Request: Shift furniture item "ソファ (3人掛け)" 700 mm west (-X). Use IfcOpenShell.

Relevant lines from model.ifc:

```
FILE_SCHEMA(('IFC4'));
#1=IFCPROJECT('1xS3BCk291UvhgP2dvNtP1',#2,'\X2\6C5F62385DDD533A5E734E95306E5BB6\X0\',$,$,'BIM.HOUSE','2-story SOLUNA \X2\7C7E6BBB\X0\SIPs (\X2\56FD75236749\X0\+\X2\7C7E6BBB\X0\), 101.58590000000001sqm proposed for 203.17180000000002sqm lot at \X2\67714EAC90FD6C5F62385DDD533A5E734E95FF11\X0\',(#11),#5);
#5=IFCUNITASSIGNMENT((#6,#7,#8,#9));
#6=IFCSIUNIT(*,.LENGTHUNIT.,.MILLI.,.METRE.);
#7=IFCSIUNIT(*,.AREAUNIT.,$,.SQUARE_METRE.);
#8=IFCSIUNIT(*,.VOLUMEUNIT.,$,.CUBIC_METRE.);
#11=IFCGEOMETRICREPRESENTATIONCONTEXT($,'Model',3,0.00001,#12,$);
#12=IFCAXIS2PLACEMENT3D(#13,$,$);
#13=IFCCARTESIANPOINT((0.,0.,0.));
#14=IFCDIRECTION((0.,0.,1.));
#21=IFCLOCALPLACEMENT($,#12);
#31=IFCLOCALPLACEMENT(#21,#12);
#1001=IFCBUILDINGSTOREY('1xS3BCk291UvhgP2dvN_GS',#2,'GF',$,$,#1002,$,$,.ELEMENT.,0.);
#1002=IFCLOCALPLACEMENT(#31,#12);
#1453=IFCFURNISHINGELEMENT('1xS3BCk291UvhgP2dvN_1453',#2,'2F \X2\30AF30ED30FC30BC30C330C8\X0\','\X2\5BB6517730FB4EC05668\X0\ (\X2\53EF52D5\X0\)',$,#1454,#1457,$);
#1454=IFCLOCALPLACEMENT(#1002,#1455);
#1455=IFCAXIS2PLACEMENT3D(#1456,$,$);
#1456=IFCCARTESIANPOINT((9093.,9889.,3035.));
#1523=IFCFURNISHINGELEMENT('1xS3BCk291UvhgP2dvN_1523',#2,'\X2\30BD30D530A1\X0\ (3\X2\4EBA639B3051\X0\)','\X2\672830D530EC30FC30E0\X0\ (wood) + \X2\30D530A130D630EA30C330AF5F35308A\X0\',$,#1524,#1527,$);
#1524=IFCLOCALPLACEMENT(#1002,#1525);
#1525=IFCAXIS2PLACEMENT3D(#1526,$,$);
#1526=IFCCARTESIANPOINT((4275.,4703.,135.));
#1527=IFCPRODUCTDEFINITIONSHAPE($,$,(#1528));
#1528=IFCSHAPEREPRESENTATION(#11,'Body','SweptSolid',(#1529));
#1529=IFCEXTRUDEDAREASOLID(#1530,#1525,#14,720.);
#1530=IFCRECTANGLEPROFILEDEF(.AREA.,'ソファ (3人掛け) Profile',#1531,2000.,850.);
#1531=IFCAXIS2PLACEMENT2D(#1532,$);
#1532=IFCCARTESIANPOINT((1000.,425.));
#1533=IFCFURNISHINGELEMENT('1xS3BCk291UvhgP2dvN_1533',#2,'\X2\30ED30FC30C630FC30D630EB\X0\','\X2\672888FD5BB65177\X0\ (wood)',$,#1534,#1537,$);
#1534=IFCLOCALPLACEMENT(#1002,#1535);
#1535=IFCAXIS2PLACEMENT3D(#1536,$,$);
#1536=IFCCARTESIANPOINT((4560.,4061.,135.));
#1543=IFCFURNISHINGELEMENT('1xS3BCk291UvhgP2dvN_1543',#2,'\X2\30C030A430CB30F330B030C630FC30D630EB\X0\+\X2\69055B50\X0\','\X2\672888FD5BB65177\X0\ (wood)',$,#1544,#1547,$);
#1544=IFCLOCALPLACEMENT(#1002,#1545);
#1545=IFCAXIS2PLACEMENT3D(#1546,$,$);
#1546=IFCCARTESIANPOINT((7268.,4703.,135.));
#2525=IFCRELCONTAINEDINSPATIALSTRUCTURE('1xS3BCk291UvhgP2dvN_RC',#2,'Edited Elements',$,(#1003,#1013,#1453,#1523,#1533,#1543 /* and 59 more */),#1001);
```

```python
import ifcopenshell
import ifcopenshell.api.geometry
import ifcopenshell.util.placement

model = ifcopenshell.open("model.ifc")

item = model.by_guid("1xS3BCk291UvhgP2dvN_1523")
matrix = ifcopenshell.util.placement.get_local_placement(item.ObjectPlacement)
matrix[0, 3] -= 700.0
ifcopenshell.api.geometry.edit_object_placement(model, product=item, matrix=matrix, is_si=False)

print(ifcopenshell.util.placement.get_local_placement(item.ObjectPlacement).round(3) + 0.0)

model.write("model_rev.ifc")
```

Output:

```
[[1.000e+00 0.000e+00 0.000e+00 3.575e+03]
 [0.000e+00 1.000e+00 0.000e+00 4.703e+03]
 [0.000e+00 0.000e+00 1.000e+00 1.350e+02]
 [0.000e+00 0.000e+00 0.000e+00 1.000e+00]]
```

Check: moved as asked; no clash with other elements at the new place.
